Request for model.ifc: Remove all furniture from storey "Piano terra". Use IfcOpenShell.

First a look at what the model holds.

```python
import ifcopenshell
import ifcopenshell.util.element

model = ifcopenshell.open("model.ifc")
print(model.schema)
storey = next(s for s in model.by_type("IfcBuildingStorey") if s.Name == "Piano terra")
furniture = [e for e in ifcopenshell.util.element.get_decomposition(storey) if e.is_a("IfcFurnishingElement")]
seen = {}
for e in furniture:
    element_type = ifcopenshell.util.element.get_type(e)
    name = element_type.Name if element_type not in (None, e) else None
    seen[name] = seen.get(name, 0) + 1
for name, count in sorted(seen.items(), key=str):
    print(count, "x", name)
```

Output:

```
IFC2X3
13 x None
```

```python
import ifcopenshell
import ifcopenshell.api.root
import ifcopenshell.util.element

model = ifcopenshell.open("model.ifc")

storey = next(s for s in model.by_type("IfcBuildingStorey") if s.Name == "Piano terra")
furniture = [e for e in ifcopenshell.util.element.get_decomposition(storey) if e.is_a("IfcFurnishingElement")]

for e in furniture:
    ifcopenshell.api.root.remove_product(model, product=e)
print(len(furniture), "removed")

model.write("model_edited.ifc")
```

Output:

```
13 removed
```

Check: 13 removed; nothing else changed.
